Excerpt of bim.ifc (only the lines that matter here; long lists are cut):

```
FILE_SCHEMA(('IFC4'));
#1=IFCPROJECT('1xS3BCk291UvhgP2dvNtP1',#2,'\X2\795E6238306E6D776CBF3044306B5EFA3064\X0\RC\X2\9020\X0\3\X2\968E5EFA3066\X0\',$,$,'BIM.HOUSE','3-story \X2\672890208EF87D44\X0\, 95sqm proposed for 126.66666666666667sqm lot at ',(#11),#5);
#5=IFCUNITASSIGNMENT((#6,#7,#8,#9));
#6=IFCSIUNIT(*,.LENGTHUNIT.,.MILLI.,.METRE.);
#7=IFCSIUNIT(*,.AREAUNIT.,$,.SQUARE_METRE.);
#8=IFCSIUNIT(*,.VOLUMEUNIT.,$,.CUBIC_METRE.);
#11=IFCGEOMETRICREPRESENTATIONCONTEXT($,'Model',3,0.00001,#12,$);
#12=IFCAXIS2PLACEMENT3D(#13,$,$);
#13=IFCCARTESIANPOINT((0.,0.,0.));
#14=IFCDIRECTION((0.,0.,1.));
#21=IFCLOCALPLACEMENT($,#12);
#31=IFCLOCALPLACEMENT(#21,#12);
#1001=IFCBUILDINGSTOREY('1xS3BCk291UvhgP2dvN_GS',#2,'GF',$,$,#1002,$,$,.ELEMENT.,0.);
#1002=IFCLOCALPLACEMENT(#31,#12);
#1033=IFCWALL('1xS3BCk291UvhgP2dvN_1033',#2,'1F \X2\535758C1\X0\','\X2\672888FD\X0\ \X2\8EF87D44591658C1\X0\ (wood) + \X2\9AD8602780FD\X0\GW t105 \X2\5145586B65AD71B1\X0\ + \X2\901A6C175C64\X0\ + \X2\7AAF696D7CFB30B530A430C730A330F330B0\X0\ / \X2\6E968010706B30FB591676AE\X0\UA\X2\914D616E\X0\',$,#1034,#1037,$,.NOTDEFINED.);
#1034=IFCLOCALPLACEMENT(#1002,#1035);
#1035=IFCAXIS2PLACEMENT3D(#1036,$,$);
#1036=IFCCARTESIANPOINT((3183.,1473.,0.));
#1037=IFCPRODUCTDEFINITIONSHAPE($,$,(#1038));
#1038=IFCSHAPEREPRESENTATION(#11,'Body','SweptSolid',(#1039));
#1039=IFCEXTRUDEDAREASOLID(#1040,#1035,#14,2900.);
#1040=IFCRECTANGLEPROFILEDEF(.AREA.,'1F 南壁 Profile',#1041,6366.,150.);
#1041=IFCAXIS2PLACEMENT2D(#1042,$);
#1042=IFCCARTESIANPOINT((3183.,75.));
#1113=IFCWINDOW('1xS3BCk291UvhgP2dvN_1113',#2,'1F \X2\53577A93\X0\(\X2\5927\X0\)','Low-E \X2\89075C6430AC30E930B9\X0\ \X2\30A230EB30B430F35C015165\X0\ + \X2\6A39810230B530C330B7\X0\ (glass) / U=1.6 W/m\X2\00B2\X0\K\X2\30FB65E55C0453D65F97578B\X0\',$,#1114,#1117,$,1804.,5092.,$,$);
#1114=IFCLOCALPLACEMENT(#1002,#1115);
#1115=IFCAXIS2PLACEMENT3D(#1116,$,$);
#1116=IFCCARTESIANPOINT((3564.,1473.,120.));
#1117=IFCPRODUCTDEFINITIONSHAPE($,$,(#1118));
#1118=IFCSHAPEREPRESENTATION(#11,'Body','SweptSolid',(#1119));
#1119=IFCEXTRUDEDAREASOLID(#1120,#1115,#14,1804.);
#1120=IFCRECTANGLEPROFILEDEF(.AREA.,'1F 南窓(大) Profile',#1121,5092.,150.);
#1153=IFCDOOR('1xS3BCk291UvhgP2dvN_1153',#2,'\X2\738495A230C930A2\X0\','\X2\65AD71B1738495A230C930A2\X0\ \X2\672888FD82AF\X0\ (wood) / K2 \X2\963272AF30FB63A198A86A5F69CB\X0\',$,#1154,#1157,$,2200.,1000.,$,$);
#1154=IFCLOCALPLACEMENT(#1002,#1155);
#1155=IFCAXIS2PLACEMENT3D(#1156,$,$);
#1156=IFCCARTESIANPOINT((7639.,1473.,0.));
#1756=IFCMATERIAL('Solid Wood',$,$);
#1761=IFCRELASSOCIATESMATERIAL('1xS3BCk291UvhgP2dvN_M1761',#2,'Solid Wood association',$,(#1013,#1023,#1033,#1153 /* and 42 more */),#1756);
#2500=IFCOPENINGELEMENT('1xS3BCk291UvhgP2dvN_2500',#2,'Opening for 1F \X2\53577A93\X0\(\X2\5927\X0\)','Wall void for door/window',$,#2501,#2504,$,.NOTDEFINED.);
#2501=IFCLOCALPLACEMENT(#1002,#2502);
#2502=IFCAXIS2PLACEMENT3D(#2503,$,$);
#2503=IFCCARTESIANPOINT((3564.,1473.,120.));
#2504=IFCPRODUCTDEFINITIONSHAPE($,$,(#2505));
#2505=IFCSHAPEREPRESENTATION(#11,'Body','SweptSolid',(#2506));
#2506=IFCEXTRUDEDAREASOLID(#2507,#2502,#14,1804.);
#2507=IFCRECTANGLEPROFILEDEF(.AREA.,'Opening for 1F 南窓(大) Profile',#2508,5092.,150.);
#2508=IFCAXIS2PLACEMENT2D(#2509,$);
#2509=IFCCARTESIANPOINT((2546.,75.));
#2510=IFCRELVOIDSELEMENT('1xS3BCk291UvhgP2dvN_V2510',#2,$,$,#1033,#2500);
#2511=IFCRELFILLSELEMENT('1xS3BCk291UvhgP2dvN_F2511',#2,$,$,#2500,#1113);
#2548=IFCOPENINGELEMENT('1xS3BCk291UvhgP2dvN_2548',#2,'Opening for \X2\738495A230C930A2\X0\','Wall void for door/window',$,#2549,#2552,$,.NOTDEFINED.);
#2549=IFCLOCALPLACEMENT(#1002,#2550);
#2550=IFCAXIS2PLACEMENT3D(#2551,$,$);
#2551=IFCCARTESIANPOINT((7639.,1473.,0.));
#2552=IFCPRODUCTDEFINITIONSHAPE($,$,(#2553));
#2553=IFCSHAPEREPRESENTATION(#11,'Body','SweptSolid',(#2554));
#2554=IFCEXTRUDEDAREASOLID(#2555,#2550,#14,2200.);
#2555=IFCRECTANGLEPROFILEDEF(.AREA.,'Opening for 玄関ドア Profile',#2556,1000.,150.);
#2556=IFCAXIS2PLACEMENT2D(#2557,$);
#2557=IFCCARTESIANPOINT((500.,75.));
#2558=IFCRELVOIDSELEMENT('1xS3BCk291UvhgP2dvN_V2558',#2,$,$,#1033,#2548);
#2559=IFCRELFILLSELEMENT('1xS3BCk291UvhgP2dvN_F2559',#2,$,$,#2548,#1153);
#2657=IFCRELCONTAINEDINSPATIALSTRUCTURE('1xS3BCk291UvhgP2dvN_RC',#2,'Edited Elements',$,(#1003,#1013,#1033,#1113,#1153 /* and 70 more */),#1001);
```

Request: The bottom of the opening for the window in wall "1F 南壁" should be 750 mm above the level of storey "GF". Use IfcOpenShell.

```python
import numpy as np
import ifcopenshell
import ifcopenshell.api.geometry
import ifcopenshell.geom
import ifcopenshell.util.element
import ifcopenshell.util.placement
import ifcopenshell.util.shape
import ifcopenshell.util.unit

model = ifcopenshell.open("bim.ifc")
unit_scale = ifcopenshell.util.unit.calculate_unit_scale(model)

window = model.by_guid("1xS3BCk291UvhgP2dvN_1113")
opening = window.FillsVoids[0].RelatingOpeningElement
storey = ifcopenshell.util.element.get_container(window, ifc_class="IfcBuildingStorey")
level = ifcopenshell.util.placement.get_local_placement(storey.ObjectPlacement)[2, 3]

# The opening's origin need not be at the sill, so measure its lowest point.
shape = ifcopenshell.geom.create_shape(ifcopenshell.geom.settings(), opening)
bottom = ifcopenshell.util.shape.get_shape_bottom_elevation(shape, shape.geometry) / unit_scale
dz = level + 0.75 / unit_scale - bottom

shift = np.array([0.0, 0.0, dz])
# The window is not placed relative to its opening, so move both.
for product in (opening, window):
    matrix = ifcopenshell.util.placement.get_local_placement(product.ObjectPlacement)
    matrix[:3, 3] += shift
    ifcopenshell.api.geometry.edit_object_placement(model, product=product, matrix=matrix, is_si=False)

print(f"moved by {dz * unit_scale:+.3f} m")

model.write("bim_v2.ifc")
```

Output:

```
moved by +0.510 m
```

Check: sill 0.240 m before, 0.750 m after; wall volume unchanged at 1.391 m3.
